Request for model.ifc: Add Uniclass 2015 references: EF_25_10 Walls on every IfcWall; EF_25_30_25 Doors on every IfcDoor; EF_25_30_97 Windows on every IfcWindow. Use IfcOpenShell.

First a look at what the model holds.

```python
import ifcopenshell

model = ifcopenshell.open("model.ifc")
print(model.schema)
print("classifications:", [c.Name for c in model.by_type("IfcClassification")])
for ifc_class in ("IfcDoor", "IfcRoof", "IfcStair", "IfcWall", "IfcWindow"):
    print(ifc_class, len(model.by_type(ifc_class)))
```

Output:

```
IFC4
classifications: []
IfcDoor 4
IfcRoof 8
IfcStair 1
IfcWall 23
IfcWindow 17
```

```python
import ifcopenshell
import ifcopenshell.api.classification

model = ifcopenshell.open("model.ifc")

system = ifcopenshell.api.classification.add_classification(model, classification="Uniclass 2015")

codes = {
    "IfcWall": ("EF_25_10", "Walls"),
    "IfcDoor": ("EF_25_30_25", "Doors"),
    "IfcWindow": ("EF_25_30_97", "Windows"),
}
for ifc_class, (code, name) in codes.items():
    products = model.by_type(ifc_class)
    ifcopenshell.api.classification.add_reference(
        model, products=products, classification=system, identification=code, name=name
    )
    print(code, len(products))

model.write("model_updated.ifc")
```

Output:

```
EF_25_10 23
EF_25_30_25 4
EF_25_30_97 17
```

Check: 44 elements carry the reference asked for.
